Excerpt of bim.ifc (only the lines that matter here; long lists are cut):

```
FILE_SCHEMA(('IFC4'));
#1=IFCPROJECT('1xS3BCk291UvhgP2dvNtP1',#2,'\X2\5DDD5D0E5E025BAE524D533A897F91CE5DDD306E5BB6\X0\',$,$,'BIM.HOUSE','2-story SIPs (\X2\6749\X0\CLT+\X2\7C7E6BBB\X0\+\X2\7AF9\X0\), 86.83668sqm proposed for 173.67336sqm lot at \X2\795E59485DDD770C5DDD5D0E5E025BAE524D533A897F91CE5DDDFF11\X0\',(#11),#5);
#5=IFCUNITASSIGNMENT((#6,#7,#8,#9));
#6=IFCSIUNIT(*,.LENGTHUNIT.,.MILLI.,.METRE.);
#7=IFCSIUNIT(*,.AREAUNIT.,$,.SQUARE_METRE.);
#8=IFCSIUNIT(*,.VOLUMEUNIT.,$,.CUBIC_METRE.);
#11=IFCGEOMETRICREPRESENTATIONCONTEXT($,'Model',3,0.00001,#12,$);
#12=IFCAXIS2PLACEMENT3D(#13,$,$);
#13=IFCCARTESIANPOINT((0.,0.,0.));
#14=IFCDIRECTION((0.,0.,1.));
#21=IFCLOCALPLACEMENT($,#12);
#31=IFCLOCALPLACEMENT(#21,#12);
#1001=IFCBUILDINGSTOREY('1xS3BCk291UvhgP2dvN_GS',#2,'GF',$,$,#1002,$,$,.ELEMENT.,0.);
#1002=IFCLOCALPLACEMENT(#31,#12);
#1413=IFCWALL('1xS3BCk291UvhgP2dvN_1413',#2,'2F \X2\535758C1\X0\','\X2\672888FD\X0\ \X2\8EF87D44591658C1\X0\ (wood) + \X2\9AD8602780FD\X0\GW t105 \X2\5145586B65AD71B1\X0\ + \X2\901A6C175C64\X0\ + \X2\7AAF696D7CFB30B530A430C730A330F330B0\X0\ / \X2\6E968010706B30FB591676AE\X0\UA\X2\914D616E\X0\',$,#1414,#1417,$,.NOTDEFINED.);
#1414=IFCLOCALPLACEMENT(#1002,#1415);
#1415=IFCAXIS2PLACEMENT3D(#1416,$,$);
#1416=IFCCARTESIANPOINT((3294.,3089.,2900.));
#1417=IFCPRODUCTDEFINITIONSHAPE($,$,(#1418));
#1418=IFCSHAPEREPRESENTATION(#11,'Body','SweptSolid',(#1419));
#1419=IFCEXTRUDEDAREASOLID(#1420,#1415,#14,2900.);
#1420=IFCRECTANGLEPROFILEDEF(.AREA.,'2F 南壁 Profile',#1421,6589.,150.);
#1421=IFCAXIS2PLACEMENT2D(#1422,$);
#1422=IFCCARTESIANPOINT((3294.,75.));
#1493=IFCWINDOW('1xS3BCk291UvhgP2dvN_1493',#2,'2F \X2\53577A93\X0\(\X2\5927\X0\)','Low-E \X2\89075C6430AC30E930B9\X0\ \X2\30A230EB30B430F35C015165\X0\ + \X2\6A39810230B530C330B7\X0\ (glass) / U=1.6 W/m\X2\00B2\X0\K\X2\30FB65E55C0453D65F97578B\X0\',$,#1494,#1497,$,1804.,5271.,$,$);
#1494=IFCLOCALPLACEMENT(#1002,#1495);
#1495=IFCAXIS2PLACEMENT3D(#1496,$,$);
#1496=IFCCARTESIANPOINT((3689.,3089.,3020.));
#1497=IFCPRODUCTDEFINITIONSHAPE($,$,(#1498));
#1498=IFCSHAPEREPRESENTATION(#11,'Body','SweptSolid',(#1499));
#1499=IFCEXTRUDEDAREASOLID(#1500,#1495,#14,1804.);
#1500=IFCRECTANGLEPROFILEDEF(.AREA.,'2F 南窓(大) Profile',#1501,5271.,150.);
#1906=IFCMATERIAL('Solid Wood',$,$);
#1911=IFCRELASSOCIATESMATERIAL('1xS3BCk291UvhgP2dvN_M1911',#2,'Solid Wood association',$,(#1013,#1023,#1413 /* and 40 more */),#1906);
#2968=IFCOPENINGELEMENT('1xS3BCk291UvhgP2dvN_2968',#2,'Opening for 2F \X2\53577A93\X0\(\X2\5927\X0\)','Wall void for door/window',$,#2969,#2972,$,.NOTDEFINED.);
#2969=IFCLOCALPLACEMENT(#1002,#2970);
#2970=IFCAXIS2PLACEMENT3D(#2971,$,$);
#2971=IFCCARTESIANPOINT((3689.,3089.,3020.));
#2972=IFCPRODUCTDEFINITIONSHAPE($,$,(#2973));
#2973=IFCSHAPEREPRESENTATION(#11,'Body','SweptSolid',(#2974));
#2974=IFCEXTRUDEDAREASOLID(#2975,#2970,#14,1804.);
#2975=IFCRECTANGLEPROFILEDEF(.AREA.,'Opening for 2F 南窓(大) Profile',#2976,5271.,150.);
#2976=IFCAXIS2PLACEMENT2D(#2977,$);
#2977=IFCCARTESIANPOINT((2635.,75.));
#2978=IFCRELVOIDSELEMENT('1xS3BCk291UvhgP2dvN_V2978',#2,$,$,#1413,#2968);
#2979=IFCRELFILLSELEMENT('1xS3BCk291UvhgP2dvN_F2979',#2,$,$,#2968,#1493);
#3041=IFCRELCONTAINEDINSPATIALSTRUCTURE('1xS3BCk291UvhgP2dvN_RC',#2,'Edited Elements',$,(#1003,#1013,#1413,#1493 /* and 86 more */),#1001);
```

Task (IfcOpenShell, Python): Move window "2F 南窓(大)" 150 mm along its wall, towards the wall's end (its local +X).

```python
import ifcopenshell
import ifcopenshell.api.geometry
import ifcopenshell.util.placement

model = ifcopenshell.open("bim.ifc")

window = model.by_id(1493)
opening = window.FillsVoids[0].RelatingOpeningElement
wall = opening.VoidsElements[0].RelatingBuildingElement

wall_matrix = ifcopenshell.util.placement.get_local_placement(wall.ObjectPlacement)
shift = wall_matrix[:3, 0] * 150.0
before = ifcopenshell.util.placement.get_local_placement(window.ObjectPlacement)[:3, 3].copy()

# The window is not placed relative to its opening, so move both.
for product in (opening, window):
    matrix = ifcopenshell.util.placement.get_local_placement(product.ObjectPlacement)
    matrix[:3, 3] += shift
    ifcopenshell.api.geometry.edit_object_placement(model, product=product, matrix=matrix, is_si=False)

after = ifcopenshell.util.placement.get_local_placement(window.ObjectPlacement)[:3, 3]
print("window moved by", (after - before).round(3) + 0.0)

model.write("bim-out.ifc")
```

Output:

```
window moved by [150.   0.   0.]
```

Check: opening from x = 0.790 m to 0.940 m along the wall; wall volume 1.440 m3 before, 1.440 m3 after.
